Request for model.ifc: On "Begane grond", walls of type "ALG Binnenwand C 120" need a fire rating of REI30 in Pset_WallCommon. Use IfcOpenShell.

First a look at what the model holds.

```python
import ifcopenshell
import ifcopenshell.util.element

model = ifcopenshell.open("model.ifc")
print(model.schema)
storey = next(s for s in model.by_type("IfcBuildingStorey") if s.Name == "Begane grond")
walls = [e for e in ifcopenshell.util.element.get_decomposition(storey) if e.is_a("IfcWall")]
seen = {}
for e in walls:
    element_type = ifcopenshell.util.element.get_type(e)
    key = (element_type.Name if element_type != e and element_type else None, ifcopenshell.util.element.get_pset(e, "Pset_WallCommon", "FireRating"))
    seen[key] = seen.get(key, 0) + 1
for (name, value), count in sorted(seen.items(), key=str):
    print(count, "x", name, "|", value)
```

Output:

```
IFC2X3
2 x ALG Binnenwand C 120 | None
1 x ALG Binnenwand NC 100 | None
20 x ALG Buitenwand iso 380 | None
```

```python
import ifcopenshell
import ifcopenshell.api.pset
import ifcopenshell.util.element

model = ifcopenshell.open("model.ifc")

storey = next(s for s in model.by_type("IfcBuildingStorey") if s.Name == "Begane grond")
walls = [e for e in ifcopenshell.util.element.get_decomposition(storey) if e.is_a("IfcWall")]

count = 0
for e in walls:
    element_type = ifcopenshell.util.element.get_type(e)
    if element_type in (None, e) or element_type.Name != "ALG Binnenwand C 120":
        continue
    # add_pset returns the element's existing set when there is one.
    pset = ifcopenshell.api.pset.add_pset(model, product=e, name="Pset_WallCommon")
    ifcopenshell.api.pset.edit_pset(model, pset=pset, properties={"FireRating": "REI30"})
    count += 1

print(count, "walls updated")

model.write("model_v2.ifc")
```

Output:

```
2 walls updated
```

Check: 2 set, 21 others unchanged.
